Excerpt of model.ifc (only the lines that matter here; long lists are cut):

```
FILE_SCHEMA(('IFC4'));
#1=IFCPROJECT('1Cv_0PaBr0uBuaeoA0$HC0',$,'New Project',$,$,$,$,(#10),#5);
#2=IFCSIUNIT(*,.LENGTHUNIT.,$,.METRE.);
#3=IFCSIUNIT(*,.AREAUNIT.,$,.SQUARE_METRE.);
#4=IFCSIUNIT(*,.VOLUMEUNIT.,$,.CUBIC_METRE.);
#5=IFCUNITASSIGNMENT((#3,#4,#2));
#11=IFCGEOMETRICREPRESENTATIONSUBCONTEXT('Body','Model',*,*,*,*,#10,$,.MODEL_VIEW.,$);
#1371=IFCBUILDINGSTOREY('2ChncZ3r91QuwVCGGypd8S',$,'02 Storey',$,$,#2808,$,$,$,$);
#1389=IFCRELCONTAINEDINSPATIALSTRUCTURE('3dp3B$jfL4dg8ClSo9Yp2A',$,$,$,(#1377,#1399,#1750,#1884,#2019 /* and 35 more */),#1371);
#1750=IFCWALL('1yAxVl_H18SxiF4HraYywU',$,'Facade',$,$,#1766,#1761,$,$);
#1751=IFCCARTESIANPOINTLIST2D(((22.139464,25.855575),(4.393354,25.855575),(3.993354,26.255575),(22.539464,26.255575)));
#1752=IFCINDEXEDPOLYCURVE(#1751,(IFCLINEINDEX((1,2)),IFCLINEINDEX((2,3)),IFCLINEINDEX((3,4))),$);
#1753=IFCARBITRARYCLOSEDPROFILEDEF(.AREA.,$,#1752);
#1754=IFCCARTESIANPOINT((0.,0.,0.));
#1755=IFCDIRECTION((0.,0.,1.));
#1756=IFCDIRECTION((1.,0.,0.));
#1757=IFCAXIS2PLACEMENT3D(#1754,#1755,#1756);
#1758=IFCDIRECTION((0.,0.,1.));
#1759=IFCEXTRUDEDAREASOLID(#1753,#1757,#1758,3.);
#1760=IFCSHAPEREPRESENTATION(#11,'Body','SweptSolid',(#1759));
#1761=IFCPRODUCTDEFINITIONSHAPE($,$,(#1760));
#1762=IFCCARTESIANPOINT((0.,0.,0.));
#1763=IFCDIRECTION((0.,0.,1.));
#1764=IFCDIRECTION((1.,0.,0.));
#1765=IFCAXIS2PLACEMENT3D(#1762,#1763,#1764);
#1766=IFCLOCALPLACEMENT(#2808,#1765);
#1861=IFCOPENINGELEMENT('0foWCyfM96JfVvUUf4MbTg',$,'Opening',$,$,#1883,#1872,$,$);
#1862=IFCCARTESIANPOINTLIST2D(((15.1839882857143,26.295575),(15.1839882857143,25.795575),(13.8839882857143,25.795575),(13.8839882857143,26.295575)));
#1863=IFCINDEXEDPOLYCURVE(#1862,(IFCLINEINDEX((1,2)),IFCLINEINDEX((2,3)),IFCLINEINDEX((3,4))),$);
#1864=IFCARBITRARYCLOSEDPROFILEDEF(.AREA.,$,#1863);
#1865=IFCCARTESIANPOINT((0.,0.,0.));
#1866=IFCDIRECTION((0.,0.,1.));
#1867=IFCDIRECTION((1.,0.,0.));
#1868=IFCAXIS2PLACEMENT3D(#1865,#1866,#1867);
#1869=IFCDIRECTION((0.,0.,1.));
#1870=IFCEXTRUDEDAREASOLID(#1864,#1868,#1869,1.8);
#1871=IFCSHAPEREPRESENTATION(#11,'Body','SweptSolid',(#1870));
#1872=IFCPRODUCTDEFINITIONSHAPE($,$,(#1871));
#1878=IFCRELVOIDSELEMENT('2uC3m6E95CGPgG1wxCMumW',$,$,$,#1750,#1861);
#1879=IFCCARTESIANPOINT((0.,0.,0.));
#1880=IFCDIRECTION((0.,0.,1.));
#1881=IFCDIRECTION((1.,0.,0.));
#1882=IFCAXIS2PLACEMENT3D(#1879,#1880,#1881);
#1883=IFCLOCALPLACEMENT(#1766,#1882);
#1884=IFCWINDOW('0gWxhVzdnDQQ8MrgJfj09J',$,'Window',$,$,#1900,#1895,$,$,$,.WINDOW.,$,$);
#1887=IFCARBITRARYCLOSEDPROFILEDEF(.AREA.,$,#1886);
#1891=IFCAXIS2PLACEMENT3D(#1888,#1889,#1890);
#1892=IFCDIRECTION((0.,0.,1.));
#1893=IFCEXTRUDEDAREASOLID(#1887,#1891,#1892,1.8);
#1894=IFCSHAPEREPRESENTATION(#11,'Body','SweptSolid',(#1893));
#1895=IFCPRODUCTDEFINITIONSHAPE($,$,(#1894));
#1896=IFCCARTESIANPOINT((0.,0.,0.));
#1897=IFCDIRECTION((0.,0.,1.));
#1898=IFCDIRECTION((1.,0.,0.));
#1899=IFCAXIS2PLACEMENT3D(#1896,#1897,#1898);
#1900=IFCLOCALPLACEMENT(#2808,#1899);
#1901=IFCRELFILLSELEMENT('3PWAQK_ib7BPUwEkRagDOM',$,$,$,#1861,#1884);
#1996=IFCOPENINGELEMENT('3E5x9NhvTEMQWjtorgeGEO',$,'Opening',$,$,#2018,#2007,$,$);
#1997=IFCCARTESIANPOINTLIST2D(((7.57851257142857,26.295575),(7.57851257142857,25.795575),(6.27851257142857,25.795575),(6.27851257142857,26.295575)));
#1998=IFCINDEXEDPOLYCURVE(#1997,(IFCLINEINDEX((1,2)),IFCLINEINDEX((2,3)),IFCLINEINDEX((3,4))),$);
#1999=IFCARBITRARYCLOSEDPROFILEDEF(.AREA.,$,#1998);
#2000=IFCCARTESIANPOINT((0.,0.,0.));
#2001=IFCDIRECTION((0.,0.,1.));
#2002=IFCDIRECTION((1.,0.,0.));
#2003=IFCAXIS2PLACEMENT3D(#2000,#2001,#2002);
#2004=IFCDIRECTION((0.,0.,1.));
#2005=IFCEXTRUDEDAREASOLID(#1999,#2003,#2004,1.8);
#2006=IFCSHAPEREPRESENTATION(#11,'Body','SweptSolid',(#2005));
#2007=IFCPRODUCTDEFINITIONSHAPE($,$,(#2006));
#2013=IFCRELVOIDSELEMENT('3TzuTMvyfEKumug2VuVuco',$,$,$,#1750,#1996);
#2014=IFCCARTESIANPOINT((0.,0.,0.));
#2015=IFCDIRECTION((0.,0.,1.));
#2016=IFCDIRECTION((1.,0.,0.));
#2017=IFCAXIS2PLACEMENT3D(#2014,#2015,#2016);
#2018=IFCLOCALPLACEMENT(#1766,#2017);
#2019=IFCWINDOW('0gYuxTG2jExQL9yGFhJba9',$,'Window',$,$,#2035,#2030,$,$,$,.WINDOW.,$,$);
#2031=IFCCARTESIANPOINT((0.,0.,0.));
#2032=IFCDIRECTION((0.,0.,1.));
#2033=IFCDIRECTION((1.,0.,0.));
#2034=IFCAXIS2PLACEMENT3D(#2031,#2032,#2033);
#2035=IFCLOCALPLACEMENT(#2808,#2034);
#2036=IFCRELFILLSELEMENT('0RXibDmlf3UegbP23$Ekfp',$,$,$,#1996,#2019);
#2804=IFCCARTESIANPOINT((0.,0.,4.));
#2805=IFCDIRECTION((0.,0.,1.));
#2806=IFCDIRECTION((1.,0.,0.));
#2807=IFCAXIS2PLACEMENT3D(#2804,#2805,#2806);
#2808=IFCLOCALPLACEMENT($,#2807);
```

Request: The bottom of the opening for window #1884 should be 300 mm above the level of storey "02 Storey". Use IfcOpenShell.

```python
import numpy as np
import ifcopenshell
import ifcopenshell.api.geometry
import ifcopenshell.geom
import ifcopenshell.util.element
import ifcopenshell.util.placement
import ifcopenshell.util.shape
import ifcopenshell.util.unit

model = ifcopenshell.open("model.ifc")
unit_scale = ifcopenshell.util.unit.calculate_unit_scale(model)

window = model.by_guid("0gWxhVzdnDQQ8MrgJfj09J")
opening = window.FillsVoids[0].RelatingOpeningElement
storey = ifcopenshell.util.element.get_container(window, ifc_class="IfcBuildingStorey")
level = ifcopenshell.util.placement.get_local_placement(storey.ObjectPlacement)[2, 3]

# The opening's origin need not be at the sill, so measure its lowest point.
shape = ifcopenshell.geom.create_shape(ifcopenshell.geom.settings(), opening)
bottom = ifcopenshell.util.shape.get_shape_bottom_elevation(shape, shape.geometry) / unit_scale
dz = level + 0.3 / unit_scale - bottom

shift = np.array([0.0, 0.0, dz])
# The window is not placed relative to its opening, so move both.
for product in (opening, window):
    matrix = ifcopenshell.util.placement.get_local_placement(product.ObjectPlacement)
    matrix[:3, 3] += shift
    ifcopenshell.api.geometry.edit_object_placement(model, product=product, matrix=matrix, is_si=False)

print(f"moved by {dz * unit_scale:+.3f} m")

model.write("model_edited.ifc")
```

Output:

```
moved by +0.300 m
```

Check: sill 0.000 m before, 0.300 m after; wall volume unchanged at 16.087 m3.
